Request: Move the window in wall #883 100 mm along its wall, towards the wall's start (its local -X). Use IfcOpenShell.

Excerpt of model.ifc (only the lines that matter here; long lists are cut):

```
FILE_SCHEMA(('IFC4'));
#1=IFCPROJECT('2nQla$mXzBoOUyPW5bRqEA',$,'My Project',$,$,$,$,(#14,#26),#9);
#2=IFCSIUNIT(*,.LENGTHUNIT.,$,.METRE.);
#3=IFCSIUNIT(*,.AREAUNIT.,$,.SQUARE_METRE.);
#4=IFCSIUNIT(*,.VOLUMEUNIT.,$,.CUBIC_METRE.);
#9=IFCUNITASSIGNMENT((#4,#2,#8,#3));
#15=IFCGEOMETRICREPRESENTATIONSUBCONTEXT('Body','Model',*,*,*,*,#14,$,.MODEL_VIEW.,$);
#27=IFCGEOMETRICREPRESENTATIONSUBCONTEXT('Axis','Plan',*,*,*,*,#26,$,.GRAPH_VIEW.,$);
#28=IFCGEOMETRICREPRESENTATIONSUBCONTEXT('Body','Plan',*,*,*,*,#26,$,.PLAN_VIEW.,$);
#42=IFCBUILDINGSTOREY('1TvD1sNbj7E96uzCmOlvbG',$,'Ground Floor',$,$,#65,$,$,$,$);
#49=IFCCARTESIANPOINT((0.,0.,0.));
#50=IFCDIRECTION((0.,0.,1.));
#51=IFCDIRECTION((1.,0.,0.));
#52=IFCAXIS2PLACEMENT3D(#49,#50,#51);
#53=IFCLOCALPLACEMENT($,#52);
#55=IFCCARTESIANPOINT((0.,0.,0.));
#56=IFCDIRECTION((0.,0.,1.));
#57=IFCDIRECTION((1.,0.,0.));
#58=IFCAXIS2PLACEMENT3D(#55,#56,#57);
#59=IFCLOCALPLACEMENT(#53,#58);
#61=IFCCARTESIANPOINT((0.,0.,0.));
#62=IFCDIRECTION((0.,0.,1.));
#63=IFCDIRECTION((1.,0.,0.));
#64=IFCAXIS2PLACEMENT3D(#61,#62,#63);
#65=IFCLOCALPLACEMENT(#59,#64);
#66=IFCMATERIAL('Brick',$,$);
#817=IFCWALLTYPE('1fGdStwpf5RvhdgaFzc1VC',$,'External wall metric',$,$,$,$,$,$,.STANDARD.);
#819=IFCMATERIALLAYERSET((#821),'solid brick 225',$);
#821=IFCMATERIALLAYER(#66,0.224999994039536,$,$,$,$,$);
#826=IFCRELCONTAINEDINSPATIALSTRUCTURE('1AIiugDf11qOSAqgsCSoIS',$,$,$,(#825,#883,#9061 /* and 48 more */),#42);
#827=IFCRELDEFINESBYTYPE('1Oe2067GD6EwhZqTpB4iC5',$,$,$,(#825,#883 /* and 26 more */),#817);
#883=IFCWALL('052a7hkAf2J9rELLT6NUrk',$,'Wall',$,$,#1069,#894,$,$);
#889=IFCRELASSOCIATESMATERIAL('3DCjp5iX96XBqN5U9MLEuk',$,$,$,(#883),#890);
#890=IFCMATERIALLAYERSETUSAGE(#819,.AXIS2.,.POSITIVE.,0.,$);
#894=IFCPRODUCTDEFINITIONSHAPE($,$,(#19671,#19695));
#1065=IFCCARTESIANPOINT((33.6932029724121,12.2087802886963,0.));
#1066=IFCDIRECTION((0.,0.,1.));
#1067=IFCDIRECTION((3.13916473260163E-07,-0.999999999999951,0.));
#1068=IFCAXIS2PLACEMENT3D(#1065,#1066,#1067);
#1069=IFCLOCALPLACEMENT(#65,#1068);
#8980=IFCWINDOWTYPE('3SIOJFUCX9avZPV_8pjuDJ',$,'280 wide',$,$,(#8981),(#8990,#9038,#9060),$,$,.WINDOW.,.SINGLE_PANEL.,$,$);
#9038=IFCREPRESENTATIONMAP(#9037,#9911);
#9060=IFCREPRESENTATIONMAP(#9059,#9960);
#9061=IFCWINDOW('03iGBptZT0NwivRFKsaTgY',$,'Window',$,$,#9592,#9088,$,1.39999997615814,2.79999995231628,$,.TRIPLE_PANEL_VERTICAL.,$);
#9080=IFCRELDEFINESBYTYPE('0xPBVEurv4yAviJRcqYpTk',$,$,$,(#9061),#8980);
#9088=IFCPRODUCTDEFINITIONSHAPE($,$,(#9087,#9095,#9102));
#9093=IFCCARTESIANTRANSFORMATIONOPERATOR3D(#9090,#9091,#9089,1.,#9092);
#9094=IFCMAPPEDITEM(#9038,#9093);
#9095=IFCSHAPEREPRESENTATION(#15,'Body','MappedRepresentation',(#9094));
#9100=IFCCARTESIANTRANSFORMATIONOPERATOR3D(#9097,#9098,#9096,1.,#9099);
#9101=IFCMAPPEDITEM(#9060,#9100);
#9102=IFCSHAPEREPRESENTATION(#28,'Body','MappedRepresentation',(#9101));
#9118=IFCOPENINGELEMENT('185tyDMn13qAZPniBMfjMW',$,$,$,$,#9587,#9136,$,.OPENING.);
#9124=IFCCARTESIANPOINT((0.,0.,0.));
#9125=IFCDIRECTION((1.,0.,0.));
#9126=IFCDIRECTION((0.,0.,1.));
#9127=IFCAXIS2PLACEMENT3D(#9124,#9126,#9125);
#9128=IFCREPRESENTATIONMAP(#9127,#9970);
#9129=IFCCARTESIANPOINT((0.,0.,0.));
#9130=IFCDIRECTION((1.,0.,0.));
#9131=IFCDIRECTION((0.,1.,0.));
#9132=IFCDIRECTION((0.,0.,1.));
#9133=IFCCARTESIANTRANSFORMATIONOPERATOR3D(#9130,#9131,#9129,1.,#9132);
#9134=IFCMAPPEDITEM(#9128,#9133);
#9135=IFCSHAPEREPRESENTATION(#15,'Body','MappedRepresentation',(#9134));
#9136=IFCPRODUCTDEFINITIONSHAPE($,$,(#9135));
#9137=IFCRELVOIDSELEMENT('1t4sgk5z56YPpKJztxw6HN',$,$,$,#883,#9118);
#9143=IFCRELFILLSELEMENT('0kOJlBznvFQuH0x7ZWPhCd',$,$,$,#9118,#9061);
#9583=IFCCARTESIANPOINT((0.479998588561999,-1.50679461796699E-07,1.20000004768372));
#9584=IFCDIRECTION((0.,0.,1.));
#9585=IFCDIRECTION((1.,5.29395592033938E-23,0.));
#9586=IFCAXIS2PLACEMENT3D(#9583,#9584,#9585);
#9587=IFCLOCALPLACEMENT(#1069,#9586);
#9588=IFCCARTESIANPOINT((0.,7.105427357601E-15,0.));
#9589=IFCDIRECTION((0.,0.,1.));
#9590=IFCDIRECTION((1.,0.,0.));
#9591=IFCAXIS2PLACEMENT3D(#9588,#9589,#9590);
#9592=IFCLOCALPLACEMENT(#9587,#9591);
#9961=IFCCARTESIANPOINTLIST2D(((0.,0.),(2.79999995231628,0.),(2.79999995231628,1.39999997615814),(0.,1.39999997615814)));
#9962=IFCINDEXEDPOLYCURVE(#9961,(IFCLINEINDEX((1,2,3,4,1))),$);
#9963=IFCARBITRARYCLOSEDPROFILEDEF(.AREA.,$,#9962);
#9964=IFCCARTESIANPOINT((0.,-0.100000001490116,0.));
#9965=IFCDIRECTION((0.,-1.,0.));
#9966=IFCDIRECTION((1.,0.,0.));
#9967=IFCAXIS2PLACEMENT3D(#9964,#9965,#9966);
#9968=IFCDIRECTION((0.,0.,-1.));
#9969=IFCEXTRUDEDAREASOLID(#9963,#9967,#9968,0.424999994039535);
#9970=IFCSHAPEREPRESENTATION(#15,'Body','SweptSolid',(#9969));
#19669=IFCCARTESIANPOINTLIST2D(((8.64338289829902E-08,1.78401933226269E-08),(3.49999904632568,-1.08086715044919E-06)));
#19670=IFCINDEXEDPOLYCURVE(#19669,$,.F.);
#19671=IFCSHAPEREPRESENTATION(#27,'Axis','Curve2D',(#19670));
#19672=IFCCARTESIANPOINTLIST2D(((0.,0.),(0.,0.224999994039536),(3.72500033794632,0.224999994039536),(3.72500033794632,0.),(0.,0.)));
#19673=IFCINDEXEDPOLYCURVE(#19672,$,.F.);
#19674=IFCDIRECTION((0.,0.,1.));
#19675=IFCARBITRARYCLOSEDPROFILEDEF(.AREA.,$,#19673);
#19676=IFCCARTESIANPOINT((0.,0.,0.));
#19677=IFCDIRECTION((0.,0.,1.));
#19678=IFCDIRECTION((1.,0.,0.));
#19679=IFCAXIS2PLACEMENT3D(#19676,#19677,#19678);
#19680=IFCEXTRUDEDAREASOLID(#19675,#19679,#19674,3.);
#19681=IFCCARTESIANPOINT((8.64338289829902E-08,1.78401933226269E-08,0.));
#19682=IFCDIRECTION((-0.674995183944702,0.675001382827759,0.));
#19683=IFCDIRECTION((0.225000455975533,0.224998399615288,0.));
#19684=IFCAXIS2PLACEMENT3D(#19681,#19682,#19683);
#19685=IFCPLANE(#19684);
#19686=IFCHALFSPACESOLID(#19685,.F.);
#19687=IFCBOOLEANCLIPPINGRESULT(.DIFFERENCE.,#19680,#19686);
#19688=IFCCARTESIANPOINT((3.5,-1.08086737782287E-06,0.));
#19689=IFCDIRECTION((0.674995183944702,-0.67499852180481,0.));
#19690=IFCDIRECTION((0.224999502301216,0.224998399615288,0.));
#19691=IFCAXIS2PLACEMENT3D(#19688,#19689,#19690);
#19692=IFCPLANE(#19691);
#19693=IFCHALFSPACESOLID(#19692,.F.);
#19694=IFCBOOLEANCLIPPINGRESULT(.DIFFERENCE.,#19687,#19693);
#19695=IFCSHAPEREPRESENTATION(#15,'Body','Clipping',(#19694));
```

```python
import ifcopenshell
import ifcopenshell.api.geometry
import ifcopenshell.util.placement

model = ifcopenshell.open("model.ifc")

window = model.by_id(9061)
opening = window.FillsVoids[0].RelatingOpeningElement
wall = opening.VoidsElements[0].RelatingBuildingElement

wall_matrix = ifcopenshell.util.placement.get_local_placement(wall.ObjectPlacement)
shift = wall_matrix[:3, 0] * -0.1
before = ifcopenshell.util.placement.get_local_placement(window.ObjectPlacement)[:3, 3].copy()

# The window is placed relative to its opening, so it follows when the opening moves.
matrix = ifcopenshell.util.placement.get_local_placement(opening.ObjectPlacement)
matrix[:3, 3] += shift
ifcopenshell.api.geometry.edit_object_placement(
    model, product=opening, matrix=matrix, is_si=False, should_transform_children=True
)

after = ifcopenshell.util.placement.get_local_placement(window.ObjectPlacement)[:3, 3]
print("window moved by", (after - before).round(3) + 0.0)

model.write("model_v2.ifc")
```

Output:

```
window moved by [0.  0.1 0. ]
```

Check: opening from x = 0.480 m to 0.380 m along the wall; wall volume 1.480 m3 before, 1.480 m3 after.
